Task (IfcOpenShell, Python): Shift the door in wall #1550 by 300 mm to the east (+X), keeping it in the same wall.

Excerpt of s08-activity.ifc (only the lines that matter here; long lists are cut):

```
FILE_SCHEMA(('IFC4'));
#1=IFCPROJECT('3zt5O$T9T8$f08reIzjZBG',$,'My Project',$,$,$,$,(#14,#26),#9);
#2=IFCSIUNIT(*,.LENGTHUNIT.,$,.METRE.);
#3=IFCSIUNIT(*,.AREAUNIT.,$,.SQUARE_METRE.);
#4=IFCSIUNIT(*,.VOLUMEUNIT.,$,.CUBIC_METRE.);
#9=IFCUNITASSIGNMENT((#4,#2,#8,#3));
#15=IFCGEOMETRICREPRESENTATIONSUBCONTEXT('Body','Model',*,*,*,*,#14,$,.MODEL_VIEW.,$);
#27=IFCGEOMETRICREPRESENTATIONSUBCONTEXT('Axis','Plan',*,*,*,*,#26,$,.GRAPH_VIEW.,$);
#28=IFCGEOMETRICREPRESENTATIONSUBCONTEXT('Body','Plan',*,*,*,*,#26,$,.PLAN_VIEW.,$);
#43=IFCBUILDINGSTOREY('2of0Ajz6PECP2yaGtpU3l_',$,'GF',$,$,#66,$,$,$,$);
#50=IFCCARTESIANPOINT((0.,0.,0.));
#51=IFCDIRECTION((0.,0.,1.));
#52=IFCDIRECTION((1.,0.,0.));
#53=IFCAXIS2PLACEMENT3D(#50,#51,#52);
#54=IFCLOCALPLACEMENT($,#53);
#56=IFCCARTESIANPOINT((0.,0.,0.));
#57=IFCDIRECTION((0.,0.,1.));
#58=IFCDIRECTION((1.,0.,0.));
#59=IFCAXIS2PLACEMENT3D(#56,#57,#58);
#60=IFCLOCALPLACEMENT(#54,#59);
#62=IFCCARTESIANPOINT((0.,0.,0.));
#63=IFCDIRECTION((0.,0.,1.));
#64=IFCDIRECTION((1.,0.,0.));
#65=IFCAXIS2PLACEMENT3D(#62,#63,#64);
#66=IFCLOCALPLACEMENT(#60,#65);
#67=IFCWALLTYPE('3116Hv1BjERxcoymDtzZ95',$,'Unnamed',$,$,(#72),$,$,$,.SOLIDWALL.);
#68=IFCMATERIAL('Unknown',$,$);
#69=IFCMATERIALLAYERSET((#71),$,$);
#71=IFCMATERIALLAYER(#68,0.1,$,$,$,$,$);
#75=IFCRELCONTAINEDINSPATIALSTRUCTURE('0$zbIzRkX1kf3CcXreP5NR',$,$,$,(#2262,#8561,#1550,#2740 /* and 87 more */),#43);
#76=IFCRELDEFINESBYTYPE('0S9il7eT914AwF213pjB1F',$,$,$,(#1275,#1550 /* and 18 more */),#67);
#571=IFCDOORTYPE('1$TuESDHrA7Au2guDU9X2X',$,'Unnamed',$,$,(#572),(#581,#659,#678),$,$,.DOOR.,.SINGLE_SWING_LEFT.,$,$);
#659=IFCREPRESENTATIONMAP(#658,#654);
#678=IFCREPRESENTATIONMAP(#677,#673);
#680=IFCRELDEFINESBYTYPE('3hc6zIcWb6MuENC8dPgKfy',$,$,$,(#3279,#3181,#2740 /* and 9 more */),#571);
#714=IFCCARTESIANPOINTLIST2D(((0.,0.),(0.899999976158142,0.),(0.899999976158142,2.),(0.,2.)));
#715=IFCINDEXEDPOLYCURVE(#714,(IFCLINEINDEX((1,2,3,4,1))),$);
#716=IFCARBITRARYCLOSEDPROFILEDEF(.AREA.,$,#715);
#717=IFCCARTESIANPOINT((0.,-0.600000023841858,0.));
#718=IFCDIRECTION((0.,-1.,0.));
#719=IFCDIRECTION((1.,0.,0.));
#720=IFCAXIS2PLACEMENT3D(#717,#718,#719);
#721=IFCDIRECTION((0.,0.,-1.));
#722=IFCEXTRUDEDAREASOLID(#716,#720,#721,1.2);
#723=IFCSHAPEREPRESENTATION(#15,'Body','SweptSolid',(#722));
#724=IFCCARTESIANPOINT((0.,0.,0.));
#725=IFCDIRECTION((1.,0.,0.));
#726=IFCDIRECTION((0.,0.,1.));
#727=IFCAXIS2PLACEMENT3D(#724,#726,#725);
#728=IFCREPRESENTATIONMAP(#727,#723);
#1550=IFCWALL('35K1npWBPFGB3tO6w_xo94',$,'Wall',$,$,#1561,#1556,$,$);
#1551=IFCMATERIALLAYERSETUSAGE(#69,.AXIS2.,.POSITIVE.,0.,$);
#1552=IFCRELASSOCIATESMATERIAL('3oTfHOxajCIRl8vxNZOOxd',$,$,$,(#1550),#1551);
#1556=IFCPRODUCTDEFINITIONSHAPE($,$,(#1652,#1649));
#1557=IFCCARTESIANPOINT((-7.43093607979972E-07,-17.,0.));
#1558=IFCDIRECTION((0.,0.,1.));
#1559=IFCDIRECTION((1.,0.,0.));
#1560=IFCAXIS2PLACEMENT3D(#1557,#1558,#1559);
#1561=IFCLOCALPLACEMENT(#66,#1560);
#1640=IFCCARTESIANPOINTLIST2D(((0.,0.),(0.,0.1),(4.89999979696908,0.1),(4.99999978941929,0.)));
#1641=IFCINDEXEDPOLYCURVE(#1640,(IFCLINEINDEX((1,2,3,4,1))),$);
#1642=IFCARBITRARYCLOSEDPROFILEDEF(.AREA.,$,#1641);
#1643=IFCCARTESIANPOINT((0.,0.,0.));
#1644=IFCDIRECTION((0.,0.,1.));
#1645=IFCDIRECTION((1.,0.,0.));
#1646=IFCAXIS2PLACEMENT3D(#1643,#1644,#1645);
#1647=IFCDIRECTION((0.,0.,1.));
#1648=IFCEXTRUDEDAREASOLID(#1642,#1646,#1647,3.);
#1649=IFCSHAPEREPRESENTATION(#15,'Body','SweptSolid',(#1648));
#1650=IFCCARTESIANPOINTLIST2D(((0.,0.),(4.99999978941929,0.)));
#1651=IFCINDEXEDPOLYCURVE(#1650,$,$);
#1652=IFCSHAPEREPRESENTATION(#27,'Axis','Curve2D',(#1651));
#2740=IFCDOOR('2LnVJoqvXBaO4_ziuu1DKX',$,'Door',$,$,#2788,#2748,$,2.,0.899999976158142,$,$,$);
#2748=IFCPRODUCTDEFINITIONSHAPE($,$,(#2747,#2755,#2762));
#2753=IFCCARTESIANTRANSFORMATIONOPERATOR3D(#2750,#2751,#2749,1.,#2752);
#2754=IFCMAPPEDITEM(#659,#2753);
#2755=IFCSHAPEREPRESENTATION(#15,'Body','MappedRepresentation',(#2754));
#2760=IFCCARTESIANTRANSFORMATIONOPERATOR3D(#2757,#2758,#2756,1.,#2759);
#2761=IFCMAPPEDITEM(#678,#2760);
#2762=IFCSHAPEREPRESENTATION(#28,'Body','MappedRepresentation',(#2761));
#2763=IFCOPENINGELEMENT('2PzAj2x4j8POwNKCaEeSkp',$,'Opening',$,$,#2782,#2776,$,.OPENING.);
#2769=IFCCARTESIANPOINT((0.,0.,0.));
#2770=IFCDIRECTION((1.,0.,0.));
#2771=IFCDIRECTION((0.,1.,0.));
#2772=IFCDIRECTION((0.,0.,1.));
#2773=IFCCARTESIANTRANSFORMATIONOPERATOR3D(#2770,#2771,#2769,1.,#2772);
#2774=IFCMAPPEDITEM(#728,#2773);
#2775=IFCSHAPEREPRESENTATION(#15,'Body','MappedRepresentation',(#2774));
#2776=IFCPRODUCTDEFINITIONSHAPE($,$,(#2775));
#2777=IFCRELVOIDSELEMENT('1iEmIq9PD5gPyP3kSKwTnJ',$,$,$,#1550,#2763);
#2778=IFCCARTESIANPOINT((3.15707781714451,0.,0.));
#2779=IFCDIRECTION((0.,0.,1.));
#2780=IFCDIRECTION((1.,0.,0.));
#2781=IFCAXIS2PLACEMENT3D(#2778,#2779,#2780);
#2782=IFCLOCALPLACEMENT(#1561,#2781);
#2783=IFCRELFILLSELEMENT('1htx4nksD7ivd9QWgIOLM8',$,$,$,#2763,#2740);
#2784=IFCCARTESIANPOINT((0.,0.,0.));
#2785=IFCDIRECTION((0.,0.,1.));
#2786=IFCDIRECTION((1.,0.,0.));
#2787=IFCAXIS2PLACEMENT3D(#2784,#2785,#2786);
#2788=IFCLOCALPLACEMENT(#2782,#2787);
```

```python
import ifcopenshell
import ifcopenshell.api.geometry
import ifcopenshell.util.placement
import ifcopenshell.util.unit

model = ifcopenshell.open("s08-activity.ifc")
unit_scale = ifcopenshell.util.unit.calculate_unit_scale(model)

door = model.by_guid("2LnVJoqvXBaO4_ziuu1DKX")
opening = door.FillsVoids[0].RelatingOpeningElement
wall = opening.VoidsElements[0].RelatingBuildingElement

wall_matrix = ifcopenshell.util.placement.get_local_placement(wall.ObjectPlacement)
shift = wall_matrix[:3, 0] * 0.3 / unit_scale
before = ifcopenshell.util.placement.get_local_placement(door.ObjectPlacement)[:3, 3].copy()

# The door is placed relative to its opening, so it follows when the opening moves.
matrix = ifcopenshell.util.placement.get_local_placement(opening.ObjectPlacement)
matrix[:3, 3] += shift
ifcopenshell.api.geometry.edit_object_placement(
    model, product=opening, matrix=matrix, is_si=False, should_transform_children=True
)

after = ifcopenshell.util.placement.get_local_placement(door.ObjectPlacement)[:3, 3]
print("door moved by", (after - before).round(3) + 0.0)

model.write("s08-activity_updated.ifc")
```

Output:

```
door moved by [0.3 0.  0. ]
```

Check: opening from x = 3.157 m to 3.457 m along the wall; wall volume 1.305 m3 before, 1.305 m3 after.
